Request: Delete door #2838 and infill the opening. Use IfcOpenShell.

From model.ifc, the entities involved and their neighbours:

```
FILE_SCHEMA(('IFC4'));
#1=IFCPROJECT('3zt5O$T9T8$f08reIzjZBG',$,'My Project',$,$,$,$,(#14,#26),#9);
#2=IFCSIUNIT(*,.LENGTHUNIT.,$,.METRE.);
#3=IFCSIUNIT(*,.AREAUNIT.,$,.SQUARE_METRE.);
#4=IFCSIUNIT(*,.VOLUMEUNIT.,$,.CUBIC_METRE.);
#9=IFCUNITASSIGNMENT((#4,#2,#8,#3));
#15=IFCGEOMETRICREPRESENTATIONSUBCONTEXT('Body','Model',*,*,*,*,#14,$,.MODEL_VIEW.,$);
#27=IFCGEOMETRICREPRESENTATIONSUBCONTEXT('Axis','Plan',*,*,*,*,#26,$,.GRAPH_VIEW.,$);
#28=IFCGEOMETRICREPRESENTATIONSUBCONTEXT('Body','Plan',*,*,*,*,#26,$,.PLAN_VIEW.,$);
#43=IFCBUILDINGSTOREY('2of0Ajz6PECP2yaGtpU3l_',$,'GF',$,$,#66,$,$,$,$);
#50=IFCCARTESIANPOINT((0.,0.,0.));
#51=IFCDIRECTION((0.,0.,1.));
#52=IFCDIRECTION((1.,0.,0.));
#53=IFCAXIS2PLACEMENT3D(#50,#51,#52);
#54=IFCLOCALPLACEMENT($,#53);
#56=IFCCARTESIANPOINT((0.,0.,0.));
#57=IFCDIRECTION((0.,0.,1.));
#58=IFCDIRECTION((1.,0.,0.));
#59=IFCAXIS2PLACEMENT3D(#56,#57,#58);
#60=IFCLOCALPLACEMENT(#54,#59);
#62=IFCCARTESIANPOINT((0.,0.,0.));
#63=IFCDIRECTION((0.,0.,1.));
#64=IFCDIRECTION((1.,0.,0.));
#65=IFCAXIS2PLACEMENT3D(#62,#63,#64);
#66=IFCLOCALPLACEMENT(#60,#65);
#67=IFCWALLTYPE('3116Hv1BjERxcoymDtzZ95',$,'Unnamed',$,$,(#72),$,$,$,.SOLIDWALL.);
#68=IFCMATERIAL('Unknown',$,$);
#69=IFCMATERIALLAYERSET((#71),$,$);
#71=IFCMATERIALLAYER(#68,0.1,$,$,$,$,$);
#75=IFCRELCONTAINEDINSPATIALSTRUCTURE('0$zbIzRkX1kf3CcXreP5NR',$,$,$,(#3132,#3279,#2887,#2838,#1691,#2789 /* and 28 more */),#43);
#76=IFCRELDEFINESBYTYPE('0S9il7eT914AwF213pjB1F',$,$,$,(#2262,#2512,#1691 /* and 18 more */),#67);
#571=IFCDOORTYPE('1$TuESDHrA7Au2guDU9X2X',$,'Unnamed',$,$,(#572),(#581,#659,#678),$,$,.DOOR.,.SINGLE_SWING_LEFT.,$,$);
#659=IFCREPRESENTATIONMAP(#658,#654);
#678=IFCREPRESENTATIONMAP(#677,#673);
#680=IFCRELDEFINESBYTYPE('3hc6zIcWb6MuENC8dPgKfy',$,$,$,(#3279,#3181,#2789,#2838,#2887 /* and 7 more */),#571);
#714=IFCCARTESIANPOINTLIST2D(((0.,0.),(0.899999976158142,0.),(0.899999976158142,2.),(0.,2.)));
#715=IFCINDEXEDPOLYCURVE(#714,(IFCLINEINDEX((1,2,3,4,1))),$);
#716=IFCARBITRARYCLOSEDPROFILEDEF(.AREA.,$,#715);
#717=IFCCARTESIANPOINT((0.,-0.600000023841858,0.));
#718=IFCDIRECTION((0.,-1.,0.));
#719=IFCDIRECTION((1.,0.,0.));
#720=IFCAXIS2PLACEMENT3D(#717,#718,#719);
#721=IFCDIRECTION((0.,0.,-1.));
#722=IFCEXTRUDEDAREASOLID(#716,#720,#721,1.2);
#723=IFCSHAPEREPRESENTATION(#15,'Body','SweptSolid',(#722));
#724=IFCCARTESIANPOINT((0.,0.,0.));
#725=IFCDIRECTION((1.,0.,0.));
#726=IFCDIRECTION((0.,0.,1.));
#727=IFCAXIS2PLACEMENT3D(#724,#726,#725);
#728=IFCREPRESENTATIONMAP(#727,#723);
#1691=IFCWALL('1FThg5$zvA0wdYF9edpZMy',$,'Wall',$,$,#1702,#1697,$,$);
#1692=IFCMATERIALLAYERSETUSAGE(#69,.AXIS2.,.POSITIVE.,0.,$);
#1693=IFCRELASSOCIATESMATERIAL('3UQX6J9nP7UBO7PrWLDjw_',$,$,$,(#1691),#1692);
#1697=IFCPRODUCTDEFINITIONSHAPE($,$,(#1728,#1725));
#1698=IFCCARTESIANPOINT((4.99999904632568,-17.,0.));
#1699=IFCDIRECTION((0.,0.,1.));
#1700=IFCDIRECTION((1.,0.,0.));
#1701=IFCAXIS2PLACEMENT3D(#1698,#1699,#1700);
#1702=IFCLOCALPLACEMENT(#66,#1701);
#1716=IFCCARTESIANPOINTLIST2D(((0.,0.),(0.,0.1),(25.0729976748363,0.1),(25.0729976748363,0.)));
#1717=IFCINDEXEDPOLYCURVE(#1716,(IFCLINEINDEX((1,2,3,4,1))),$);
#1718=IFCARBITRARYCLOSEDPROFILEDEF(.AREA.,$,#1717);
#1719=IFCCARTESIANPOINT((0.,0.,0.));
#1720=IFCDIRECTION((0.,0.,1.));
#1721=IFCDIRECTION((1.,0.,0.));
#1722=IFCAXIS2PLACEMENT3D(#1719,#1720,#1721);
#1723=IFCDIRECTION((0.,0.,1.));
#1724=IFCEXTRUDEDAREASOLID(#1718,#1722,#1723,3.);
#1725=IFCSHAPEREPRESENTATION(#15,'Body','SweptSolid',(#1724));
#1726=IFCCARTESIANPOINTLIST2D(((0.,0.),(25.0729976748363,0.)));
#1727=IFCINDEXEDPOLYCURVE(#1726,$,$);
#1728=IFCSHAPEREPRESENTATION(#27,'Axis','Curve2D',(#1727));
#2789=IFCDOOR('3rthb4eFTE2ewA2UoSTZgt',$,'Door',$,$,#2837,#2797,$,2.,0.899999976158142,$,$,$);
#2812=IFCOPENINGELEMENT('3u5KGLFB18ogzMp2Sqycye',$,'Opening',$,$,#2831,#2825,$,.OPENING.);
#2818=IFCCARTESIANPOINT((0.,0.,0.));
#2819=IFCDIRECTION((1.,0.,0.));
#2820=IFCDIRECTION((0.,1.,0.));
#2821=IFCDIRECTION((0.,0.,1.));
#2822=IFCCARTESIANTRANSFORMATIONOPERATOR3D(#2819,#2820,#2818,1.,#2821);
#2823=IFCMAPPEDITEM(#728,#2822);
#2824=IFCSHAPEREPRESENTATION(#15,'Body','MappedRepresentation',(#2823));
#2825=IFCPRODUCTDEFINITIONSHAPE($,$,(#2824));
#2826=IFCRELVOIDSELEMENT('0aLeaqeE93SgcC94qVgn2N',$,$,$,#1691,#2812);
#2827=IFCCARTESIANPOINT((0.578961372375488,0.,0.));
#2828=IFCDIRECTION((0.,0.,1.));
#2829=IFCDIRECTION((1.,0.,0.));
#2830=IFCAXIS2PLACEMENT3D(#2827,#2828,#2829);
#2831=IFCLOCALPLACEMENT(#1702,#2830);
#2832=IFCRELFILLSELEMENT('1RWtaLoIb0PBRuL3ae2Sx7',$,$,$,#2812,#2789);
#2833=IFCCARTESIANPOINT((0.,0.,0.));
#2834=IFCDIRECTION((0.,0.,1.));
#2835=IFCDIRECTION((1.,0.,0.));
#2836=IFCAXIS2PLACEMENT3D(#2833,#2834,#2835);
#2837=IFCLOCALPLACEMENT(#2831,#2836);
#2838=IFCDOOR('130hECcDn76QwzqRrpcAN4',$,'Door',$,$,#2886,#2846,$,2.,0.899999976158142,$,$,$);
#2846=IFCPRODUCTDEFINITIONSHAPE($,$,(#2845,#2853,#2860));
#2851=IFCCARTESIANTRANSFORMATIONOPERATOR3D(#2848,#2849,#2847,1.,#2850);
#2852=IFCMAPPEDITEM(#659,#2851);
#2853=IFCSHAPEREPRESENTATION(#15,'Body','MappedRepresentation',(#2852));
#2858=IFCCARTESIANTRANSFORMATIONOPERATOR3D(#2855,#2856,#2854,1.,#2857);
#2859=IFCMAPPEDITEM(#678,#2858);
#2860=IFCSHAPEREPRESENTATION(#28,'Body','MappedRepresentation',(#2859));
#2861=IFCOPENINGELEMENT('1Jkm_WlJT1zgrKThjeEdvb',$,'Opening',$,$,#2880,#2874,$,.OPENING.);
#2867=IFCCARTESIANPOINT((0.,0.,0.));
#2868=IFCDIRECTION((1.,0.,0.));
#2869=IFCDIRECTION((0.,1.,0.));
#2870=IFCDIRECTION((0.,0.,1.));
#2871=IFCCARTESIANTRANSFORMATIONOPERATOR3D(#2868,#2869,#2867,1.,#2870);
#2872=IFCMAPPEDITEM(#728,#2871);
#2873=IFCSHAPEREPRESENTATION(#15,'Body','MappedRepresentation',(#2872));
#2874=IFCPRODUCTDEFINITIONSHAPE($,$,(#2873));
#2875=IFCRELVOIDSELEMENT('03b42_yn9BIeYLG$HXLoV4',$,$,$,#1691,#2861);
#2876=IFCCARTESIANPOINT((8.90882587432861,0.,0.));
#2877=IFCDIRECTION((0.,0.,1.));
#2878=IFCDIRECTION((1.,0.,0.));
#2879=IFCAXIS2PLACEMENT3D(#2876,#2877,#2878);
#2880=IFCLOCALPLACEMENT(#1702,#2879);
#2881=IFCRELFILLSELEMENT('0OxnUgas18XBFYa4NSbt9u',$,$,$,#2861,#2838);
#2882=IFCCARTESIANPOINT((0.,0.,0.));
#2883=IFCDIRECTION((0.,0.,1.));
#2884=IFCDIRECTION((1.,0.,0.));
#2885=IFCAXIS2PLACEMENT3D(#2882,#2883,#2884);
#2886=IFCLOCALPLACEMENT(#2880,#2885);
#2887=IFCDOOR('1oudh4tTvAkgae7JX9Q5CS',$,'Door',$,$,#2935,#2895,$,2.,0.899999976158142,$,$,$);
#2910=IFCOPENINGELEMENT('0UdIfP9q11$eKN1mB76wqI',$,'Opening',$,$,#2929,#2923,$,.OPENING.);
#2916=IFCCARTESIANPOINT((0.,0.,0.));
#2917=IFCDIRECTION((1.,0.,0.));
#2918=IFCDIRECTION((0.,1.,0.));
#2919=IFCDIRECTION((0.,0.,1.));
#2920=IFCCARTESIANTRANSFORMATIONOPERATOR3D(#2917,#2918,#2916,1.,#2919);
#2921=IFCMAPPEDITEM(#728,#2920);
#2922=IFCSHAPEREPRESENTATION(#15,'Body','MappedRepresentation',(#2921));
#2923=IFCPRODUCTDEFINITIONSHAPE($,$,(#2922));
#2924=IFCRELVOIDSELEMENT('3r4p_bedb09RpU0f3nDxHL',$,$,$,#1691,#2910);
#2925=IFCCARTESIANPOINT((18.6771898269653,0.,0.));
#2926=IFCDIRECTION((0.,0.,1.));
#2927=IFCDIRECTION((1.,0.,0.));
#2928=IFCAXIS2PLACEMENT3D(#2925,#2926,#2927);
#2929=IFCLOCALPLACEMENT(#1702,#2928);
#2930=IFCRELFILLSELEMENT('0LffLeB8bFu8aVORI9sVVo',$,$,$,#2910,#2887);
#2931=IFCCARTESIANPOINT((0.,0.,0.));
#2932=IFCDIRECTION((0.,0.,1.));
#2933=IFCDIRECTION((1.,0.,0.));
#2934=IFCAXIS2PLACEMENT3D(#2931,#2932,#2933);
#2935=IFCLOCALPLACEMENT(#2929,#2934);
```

```python
import ifcopenshell
import ifcopenshell.api.feature
import ifcopenshell.api.root
import ifcopenshell.geom
import ifcopenshell.util.shape

model = ifcopenshell.open("model.ifc")
settings = ifcopenshell.geom.settings()


def volume(element):
    """Net volume in cubic metres, openings subtracted."""
    shape = ifcopenshell.geom.create_shape(settings, element)
    return ifcopenshell.util.shape.get_volume(shape.geometry)


door = model.by_guid("130hECcDn76QwzqRrpcAN4")
opening = door.FillsVoids[0].RelatingOpeningElement
wall = opening.VoidsElements[0].RelatingBuildingElement
before = volume(wall)

ifcopenshell.api.root.remove_product(model, product=door)
ifcopenshell.api.feature.remove_feature(model, feature=opening)

after = volume(wall)

print(f"wall volume {before:.3f} -> {after:.3f} m3")

model.write("model_edited.ifc")
```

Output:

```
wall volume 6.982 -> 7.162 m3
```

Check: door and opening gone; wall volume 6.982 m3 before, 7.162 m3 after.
